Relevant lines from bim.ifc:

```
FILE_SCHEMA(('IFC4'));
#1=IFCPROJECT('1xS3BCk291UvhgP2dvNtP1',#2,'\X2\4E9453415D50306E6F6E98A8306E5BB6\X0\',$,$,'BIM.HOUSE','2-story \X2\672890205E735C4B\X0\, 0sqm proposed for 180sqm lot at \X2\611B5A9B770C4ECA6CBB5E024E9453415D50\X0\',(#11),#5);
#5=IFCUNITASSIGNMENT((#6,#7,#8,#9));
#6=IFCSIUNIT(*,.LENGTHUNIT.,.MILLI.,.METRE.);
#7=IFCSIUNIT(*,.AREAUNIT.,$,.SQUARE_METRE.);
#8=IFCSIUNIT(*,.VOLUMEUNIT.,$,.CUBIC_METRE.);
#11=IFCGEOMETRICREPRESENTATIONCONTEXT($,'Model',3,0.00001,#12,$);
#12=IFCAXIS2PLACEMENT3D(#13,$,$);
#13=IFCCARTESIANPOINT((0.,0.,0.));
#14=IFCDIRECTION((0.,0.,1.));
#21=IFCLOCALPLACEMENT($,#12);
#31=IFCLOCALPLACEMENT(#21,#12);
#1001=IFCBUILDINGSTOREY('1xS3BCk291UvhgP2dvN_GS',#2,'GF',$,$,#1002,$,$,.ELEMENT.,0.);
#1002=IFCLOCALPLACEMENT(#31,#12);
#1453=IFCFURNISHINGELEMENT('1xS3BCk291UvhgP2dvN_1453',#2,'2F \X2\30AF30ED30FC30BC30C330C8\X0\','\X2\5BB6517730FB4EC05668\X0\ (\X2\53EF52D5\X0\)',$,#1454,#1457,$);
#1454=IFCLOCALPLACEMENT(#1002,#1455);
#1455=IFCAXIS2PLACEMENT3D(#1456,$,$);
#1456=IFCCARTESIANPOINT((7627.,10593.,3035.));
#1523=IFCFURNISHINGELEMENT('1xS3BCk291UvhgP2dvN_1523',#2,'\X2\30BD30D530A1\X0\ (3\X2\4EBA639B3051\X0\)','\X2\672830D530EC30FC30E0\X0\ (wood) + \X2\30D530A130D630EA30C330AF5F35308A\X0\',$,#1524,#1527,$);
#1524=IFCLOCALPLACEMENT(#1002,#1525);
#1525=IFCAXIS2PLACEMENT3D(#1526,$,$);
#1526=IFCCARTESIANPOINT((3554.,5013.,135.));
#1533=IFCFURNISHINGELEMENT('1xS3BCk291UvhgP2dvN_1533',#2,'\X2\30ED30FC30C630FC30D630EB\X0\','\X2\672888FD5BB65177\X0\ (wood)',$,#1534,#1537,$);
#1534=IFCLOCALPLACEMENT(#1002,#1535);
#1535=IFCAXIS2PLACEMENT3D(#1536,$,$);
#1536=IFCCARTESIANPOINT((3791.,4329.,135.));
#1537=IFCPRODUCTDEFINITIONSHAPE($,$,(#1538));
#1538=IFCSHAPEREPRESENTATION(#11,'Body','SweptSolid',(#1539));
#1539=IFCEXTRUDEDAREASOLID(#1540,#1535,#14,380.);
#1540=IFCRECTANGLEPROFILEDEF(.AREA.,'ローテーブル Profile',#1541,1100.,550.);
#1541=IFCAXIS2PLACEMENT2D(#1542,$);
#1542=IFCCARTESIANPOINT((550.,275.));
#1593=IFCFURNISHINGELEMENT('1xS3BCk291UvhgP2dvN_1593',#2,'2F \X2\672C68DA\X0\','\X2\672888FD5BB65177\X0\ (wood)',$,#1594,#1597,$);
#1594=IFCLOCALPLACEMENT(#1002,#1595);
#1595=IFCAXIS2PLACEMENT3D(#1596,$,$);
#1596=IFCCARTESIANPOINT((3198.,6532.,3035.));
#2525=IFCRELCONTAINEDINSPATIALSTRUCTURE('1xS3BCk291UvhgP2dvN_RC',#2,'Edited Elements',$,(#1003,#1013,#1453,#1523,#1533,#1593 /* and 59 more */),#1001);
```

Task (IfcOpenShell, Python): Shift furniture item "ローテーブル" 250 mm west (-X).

```python
import ifcopenshell
import ifcopenshell.api.geometry
import ifcopenshell.util.placement

model = ifcopenshell.open("bim.ifc")

item = model.by_guid("1xS3BCk291UvhgP2dvN_1533")
matrix = ifcopenshell.util.placement.get_local_placement(item.ObjectPlacement)
matrix[0, 3] -= 250.0
ifcopenshell.api.geometry.edit_object_placement(model, product=item, matrix=matrix, is_si=False)

print(ifcopenshell.util.placement.get_local_placement(item.ObjectPlacement).round(3) + 0.0)

model.write("bim_updated.ifc")
```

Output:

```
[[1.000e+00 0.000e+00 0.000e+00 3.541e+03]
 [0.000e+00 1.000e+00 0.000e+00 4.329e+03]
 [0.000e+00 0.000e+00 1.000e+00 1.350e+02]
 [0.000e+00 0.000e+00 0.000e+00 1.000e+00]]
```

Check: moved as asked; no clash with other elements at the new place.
